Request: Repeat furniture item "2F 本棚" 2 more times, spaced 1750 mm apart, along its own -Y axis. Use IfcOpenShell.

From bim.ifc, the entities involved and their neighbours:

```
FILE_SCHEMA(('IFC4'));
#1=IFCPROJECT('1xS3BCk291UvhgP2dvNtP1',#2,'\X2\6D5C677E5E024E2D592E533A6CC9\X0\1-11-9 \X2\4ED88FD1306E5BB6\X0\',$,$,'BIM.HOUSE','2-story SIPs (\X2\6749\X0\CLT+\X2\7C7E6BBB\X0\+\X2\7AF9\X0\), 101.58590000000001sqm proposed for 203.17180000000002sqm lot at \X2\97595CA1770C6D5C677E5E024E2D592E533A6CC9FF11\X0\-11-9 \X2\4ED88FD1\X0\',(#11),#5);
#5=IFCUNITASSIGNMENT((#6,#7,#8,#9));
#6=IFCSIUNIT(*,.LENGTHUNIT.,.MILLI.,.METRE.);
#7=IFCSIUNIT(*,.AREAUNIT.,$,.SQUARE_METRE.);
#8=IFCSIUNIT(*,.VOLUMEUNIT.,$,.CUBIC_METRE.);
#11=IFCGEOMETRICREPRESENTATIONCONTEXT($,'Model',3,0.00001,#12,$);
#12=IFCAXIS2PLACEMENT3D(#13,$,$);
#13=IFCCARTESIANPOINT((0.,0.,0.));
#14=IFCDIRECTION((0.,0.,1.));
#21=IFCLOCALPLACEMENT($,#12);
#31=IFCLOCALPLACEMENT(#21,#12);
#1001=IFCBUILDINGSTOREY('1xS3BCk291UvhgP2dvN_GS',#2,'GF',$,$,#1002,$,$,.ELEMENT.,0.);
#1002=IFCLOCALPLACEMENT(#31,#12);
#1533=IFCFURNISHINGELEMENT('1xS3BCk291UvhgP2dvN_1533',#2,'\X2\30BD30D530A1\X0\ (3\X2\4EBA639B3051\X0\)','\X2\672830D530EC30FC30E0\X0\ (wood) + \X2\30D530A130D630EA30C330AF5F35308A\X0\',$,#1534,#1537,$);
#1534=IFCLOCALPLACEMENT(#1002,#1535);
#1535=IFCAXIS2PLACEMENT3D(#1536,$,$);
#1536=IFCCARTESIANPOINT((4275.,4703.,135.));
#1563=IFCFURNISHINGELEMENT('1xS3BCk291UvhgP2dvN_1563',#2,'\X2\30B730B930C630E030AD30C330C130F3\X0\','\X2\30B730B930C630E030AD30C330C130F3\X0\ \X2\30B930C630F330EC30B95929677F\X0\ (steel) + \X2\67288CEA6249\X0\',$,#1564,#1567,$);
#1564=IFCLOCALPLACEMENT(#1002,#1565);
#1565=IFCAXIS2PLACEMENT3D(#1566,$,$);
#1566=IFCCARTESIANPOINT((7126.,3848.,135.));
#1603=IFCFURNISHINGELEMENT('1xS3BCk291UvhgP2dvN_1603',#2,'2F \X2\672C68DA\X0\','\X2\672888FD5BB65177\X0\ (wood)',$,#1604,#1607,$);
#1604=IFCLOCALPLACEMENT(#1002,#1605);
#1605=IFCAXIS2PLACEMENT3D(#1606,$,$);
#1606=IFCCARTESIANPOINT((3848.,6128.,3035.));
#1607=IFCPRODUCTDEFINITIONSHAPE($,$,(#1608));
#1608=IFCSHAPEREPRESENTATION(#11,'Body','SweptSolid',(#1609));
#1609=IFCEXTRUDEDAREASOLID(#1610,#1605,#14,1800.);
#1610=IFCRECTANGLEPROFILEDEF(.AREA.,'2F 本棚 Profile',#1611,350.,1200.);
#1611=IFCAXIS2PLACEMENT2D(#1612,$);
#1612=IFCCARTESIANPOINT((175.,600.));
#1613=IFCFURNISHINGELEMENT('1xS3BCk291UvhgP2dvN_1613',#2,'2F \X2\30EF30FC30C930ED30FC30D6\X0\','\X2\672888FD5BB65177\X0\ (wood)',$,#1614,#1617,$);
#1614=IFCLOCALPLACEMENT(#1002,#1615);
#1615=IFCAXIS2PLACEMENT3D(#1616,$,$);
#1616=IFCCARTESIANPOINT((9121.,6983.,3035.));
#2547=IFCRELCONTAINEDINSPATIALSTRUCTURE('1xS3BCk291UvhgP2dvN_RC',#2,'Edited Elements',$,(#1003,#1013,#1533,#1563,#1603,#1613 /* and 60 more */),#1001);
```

```python
import ifcopenshell
import ifcopenshell.api.geometry
import ifcopenshell.api.root
import ifcopenshell.util.element
import ifcopenshell.util.placement

model = ifcopenshell.open("bim.ifc")


def reuse_history(source, copy):
    """copy_class also copies each property set's owner history, people and application; keep the originals."""
    for rel in copy.IsDefinedBy:
        if rel.is_a("IfcRelDefinesByProperties") and (history := rel.RelatingPropertyDefinition.OwnerHistory):
            rel.RelatingPropertyDefinition.OwnerHistory = source.OwnerHistory
            ifcopenshell.util.element.remove_deep2(model, history)


source = model.by_guid("1xS3BCk291UvhgP2dvN_1603")
base = ifcopenshell.util.placement.get_local_placement(source.ObjectPlacement)
step = -base[:3, 1] * 1750.0

for i in range(1, 3):
    copy = ifcopenshell.api.root.copy_class(model, product=source)
    copy.Representation = ifcopenshell.util.element.copy_deep(
        model, source.Representation, exclude=["IfcGeometricRepresentationContext", "IfcRepresentationMap"]
    )
    reuse_history(source, copy)
    matrix = base.copy()
    matrix[:3, 3] += i * step
    print("added at", matrix[:3, 3].round(3) + 0.0)
    ifcopenshell.api.geometry.edit_object_placement(model, product=copy, matrix=matrix, is_si=False)

model.write("bim_rev.ifc")
```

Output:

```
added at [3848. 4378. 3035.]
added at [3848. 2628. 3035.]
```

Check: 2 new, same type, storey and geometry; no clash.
